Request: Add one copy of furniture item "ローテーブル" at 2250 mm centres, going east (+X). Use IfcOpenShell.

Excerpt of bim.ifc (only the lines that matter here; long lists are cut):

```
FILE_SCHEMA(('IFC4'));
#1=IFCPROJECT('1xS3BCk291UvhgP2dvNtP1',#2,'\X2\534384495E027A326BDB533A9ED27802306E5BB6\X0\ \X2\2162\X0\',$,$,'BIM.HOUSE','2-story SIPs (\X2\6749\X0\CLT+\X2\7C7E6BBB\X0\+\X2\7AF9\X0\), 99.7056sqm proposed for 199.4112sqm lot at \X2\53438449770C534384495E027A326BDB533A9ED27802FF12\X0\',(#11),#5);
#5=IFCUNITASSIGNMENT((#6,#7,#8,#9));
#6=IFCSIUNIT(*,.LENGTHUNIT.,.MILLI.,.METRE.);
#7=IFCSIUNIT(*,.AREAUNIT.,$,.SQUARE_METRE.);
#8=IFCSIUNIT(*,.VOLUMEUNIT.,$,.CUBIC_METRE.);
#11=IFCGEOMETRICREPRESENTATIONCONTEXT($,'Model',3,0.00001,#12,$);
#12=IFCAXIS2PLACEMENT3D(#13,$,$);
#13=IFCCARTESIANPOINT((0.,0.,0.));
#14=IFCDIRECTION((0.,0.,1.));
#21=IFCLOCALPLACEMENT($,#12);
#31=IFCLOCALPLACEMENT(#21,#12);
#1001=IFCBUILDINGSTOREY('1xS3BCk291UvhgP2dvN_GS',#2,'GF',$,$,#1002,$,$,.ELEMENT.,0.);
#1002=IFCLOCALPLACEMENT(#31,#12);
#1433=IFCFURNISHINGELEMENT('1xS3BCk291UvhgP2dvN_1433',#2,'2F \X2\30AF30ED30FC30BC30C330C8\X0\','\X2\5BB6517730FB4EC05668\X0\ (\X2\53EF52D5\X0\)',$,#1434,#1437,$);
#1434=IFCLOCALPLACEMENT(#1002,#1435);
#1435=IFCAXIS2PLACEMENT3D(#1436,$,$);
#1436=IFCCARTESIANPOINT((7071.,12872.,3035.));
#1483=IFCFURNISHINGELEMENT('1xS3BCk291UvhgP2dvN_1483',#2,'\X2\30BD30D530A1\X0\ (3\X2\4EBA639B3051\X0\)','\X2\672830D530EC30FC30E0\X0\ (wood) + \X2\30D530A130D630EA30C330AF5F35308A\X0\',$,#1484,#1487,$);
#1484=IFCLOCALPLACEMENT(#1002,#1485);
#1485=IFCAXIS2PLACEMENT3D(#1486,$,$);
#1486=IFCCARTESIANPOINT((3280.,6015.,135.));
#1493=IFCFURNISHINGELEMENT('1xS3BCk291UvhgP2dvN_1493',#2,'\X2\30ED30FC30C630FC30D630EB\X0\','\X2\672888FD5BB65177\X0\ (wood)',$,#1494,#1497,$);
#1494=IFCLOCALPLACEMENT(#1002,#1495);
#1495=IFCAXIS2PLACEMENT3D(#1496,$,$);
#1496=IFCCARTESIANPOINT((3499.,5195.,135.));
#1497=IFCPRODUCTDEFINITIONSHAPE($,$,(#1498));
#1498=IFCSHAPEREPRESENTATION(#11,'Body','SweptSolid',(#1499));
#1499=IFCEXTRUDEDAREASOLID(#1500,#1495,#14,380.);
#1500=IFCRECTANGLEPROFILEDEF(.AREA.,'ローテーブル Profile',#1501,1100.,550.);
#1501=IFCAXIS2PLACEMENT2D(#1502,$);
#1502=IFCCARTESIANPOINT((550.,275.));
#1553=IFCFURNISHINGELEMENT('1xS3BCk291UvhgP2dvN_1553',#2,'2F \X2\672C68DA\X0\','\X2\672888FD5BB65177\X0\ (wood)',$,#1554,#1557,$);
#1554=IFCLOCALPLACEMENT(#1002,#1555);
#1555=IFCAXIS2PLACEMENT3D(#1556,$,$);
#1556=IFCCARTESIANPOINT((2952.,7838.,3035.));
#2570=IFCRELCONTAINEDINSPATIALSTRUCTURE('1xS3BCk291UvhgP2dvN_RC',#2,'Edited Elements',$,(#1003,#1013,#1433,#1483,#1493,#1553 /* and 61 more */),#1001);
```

```python
import numpy as np
import ifcopenshell
import ifcopenshell.api.geometry
import ifcopenshell.api.root
import ifcopenshell.util.element
import ifcopenshell.util.placement

model = ifcopenshell.open("bim.ifc")


def reuse_history(source, copy):
    """copy_class also copies each property set's owner history, people and application; keep the originals."""
    for rel in copy.IsDefinedBy:
        if rel.is_a("IfcRelDefinesByProperties") and (history := rel.RelatingPropertyDefinition.OwnerHistory):
            rel.RelatingPropertyDefinition.OwnerHistory = source.OwnerHistory
            ifcopenshell.util.element.remove_deep2(model, history)


source = model.by_guid("1xS3BCk291UvhgP2dvN_1493")
base = ifcopenshell.util.placement.get_local_placement(source.ObjectPlacement)
step = np.array([1.0, 0.0, 0.0]) * 2250.0

for i in range(1, 2):
    copy = ifcopenshell.api.root.copy_class(model, product=source)
    copy.Representation = ifcopenshell.util.element.copy_deep(
        model, source.Representation, exclude=["IfcGeometricRepresentationContext", "IfcRepresentationMap"]
    )
    reuse_history(source, copy)
    matrix = base.copy()
    matrix[:3, 3] += i * step
    print("added at", matrix[:3, 3].round(3) + 0.0)
    ifcopenshell.api.geometry.edit_object_placement(model, product=copy, matrix=matrix, is_si=False)

model.write("bim_v2.ifc")
```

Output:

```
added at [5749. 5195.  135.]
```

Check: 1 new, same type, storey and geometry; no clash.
